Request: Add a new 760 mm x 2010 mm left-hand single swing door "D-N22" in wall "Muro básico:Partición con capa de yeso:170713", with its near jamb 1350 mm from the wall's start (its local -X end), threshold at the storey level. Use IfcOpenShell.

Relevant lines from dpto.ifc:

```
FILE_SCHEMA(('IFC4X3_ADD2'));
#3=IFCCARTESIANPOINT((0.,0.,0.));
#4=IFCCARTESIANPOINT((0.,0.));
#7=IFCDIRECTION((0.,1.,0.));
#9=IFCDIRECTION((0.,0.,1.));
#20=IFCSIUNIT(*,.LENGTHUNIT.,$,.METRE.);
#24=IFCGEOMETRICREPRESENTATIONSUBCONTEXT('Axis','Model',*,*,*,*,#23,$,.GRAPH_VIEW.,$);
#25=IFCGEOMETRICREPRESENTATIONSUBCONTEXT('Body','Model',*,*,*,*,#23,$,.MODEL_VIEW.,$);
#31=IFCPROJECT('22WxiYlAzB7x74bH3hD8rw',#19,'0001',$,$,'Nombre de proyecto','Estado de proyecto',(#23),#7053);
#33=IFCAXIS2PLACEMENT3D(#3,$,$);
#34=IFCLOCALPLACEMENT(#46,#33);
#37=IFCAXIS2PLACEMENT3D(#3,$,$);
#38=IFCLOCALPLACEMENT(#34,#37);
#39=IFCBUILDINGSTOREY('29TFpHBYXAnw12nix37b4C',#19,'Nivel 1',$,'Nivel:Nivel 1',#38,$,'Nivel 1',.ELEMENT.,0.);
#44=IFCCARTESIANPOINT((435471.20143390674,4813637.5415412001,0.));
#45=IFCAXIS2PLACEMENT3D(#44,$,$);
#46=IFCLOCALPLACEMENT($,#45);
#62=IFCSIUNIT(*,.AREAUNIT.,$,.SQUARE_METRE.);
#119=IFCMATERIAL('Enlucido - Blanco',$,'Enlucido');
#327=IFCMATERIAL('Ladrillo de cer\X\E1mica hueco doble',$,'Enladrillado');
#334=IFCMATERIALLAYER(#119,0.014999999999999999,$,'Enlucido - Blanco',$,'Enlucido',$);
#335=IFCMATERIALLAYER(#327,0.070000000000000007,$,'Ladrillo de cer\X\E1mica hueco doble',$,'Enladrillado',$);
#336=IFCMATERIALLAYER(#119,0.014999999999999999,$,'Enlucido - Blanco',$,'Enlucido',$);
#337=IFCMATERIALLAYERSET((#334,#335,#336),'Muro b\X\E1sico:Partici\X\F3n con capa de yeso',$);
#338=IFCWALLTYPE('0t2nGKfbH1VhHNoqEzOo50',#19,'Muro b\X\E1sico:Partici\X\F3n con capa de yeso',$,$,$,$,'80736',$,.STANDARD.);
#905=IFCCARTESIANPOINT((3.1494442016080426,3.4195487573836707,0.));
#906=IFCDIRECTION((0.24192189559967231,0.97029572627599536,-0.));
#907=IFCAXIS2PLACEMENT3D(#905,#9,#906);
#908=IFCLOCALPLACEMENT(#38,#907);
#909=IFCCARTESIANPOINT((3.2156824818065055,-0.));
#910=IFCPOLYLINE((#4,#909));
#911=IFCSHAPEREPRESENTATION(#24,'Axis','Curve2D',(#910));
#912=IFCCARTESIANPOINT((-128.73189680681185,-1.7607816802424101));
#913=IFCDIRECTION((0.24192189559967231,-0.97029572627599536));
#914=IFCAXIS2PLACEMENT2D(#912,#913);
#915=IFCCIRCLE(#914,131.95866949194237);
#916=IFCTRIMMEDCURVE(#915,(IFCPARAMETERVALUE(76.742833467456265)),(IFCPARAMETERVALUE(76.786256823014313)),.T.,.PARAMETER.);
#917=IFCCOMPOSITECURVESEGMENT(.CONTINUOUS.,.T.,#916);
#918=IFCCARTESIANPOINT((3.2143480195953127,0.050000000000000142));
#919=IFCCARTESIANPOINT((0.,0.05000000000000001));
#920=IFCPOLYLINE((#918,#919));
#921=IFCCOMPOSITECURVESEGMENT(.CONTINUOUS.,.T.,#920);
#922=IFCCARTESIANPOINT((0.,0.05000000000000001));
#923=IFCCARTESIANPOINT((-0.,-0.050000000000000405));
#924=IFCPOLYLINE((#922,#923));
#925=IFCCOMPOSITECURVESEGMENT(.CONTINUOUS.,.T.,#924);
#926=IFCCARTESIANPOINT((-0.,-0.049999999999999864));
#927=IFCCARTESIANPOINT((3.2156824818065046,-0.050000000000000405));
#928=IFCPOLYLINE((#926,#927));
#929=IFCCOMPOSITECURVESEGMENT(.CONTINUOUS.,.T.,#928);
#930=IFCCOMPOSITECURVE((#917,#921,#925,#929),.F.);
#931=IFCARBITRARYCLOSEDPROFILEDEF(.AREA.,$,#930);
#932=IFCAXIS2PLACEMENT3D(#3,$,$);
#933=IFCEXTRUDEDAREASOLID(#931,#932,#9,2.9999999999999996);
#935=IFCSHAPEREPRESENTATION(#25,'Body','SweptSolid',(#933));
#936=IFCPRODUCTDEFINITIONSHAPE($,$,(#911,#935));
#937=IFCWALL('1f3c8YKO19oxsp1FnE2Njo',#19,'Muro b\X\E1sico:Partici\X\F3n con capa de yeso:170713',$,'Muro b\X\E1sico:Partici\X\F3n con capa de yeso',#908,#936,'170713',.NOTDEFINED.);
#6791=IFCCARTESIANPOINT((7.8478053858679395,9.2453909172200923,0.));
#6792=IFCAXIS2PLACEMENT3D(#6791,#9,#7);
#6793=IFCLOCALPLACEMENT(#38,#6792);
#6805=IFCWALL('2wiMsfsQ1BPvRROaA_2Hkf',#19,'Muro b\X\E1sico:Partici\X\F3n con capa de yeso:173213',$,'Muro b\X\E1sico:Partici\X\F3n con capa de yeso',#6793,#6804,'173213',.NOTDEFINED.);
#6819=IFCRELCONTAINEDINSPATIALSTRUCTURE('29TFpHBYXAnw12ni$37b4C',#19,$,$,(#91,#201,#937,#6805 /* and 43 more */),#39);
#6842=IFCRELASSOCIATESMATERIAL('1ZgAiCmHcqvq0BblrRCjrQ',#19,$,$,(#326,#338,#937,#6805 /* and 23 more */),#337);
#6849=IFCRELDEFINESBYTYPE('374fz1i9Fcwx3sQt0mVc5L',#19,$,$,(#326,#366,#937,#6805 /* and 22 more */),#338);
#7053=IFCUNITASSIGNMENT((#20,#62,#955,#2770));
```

```python
import numpy as np
import ifcopenshell
import ifcopenshell.api.feature
import ifcopenshell.api.geometry
import ifcopenshell.api.root
import ifcopenshell.api.spatial
import ifcopenshell.geom
import ifcopenshell.util.element
import ifcopenshell.util.placement
import ifcopenshell.util.representation
import ifcopenshell.util.shape
import ifcopenshell.util.unit

model = ifcopenshell.open("dpto.ifc")
unit_scale = ifcopenshell.util.unit.calculate_unit_scale(model)
settings = ifcopenshell.geom.settings()


def volume(element):
    """Net volume in cubic metres, openings subtracted."""
    shape = ifcopenshell.geom.create_shape(settings, element)
    return ifcopenshell.util.shape.get_volume(shape.geometry)


wall = model.by_guid("1f3c8YKO19oxsp1FnE2Njo")
storey = ifcopenshell.util.element.get_container(wall, ifc_class="IfcBuildingStorey")
context = ifcopenshell.util.representation.get_context(model, "Model", "Body", "MODEL_VIEW")
before = volume(wall)

width, height, from_end, sill = 0.76, 2.01, 1.35, 0.0  # metres

# The wall runs along its own X axis, and the end named is its -X end.
wall_shape = ifcopenshell.geom.create_shape(settings, wall)
x, y, z = ifcopenshell.util.shape.get_vertices(wall_shape.geometry).T
start = x.min() + from_end
face, thickness = float(y.min()), float(y.max() - y.min())
wall_matrix = ifcopenshell.util.placement.get_local_placement(wall.ObjectPlacement)
level = ifcopenshell.util.placement.get_local_placement(storey.ObjectPlacement)[2, 3]


def in_wall(x, y):
    """Placement at x, y metres in the wall's axes, at sill height."""
    matrix = wall_matrix.copy()
    matrix[:, 3] = wall_matrix @ np.array([x / unit_scale, y / unit_scale, 0.0, 1.0])
    matrix[2, 3] = level + sill / unit_scale
    return matrix


# Opening: a box that overshoots both wall faces by 50 mm.
opening = ifcopenshell.api.root.create_entity(model, ifc_class="IfcOpeningElement", predefined_type="OPENING")
box = ifcopenshell.api.geometry.add_wall_representation(
    model, context=context, length=width, height=height, thickness=thickness + 0.1
)
ifcopenshell.api.geometry.assign_representation(model, product=opening, representation=box)
ifcopenshell.api.geometry.edit_object_placement(model, product=opening, matrix=in_wall(start, face - 0.05), is_si=False)
ifcopenshell.api.feature.add_feature(model, feature=opening, element=wall)

door = ifcopenshell.api.root.create_entity(model, ifc_class="IfcDoor", name="D-N22", predefined_type="DOOR")
door.OverallWidth, door.OverallHeight = width / unit_scale, height / unit_scale
door.OperationType = "SINGLE_SWING_LEFT"
body = ifcopenshell.api.geometry.add_door_representation(
    model,
    context=context,
    overall_width=door.OverallWidth,
    overall_height=door.OverallHeight,
    operation_type="SINGLE_SWING_LEFT",
    lining_properties={"LiningDepth": thickness / unit_scale, "ThresholdDepth": thickness / unit_scale},
)
ifcopenshell.api.geometry.assign_representation(model, product=door, representation=body)
ifcopenshell.api.spatial.assign_container(model, products=[door], relating_structure=storey)
ifcopenshell.api.feature.add_filling(model, opening=opening, element=door)

# The lining spans the wall, so the door starts at the wall face.
ifcopenshell.api.geometry.edit_object_placement(model, product=door, matrix=in_wall(start, face), is_si=False)

after = volume(wall)

print(f"wall volume {before:.3f} -> {after:.3f} m3")

model.write("dpto-out.ifc")
```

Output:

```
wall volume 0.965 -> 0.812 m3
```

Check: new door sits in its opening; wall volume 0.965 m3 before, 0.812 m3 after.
